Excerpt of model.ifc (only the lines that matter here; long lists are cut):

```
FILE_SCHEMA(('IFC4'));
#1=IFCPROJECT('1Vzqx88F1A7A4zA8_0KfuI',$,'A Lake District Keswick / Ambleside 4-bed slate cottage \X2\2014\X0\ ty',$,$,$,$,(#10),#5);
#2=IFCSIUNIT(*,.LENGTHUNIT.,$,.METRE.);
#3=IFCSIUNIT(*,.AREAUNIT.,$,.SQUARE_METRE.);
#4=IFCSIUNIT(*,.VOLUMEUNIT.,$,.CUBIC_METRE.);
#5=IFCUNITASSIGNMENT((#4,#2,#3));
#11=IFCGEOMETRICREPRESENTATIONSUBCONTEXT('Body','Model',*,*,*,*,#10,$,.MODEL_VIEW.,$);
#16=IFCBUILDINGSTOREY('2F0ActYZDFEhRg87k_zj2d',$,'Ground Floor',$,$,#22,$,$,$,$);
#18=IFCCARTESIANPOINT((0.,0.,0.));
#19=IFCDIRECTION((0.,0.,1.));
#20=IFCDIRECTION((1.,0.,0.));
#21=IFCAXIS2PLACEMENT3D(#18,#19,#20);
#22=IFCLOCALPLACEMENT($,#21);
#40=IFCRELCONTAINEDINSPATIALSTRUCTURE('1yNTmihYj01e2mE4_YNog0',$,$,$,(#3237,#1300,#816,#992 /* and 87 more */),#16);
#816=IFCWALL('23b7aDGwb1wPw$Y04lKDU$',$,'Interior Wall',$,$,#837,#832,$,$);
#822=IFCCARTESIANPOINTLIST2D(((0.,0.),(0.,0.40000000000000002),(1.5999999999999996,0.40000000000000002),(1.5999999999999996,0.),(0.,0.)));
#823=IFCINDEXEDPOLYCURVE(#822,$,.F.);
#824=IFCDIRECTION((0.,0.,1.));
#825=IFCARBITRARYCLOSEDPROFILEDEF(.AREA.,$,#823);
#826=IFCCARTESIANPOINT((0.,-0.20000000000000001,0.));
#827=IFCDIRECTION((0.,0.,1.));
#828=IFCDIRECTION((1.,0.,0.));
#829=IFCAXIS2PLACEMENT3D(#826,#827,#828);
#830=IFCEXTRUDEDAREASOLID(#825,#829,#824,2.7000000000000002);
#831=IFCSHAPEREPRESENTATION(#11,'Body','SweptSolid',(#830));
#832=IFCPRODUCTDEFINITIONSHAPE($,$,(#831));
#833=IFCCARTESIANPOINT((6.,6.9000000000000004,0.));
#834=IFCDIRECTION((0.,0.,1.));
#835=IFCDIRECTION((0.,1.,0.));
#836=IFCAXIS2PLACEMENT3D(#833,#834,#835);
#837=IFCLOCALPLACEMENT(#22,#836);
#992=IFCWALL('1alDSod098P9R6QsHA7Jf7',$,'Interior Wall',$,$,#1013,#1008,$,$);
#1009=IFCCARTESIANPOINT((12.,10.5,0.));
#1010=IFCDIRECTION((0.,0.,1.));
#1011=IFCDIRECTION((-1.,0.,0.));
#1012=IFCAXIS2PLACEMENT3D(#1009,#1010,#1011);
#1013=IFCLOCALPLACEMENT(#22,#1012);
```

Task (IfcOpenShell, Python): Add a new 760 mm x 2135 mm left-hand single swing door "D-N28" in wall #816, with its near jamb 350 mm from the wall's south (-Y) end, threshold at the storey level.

```python
import numpy as np
import ifcopenshell
import ifcopenshell.api.feature
import ifcopenshell.api.geometry
import ifcopenshell.api.root
import ifcopenshell.api.spatial
import ifcopenshell.geom
import ifcopenshell.util.element
import ifcopenshell.util.placement
import ifcopenshell.util.representation
import ifcopenshell.util.shape
import ifcopenshell.util.unit

model = ifcopenshell.open("model.ifc")
unit_scale = ifcopenshell.util.unit.calculate_unit_scale(model)
settings = ifcopenshell.geom.settings()


def volume(element):
    """Net volume in cubic metres, openings subtracted."""
    shape = ifcopenshell.geom.create_shape(settings, element)
    return ifcopenshell.util.shape.get_volume(shape.geometry)


wall = model.by_guid("23b7aDGwb1wPw$Y04lKDU$")
storey = ifcopenshell.util.element.get_container(wall, ifc_class="IfcBuildingStorey")
context = ifcopenshell.util.representation.get_context(model, "Model", "Body", "MODEL_VIEW")
before = volume(wall)

width, height, from_end, sill = 0.76, 2.135, 0.35, 0.0  # metres

# The wall runs along its own X axis, and the end named is its -X end.
wall_shape = ifcopenshell.geom.create_shape(settings, wall)
x, y, z = ifcopenshell.util.shape.get_vertices(wall_shape.geometry).T
start = x.min() + from_end
face, thickness = float(y.min()), float(y.max() - y.min())
wall_matrix = ifcopenshell.util.placement.get_local_placement(wall.ObjectPlacement)
level = ifcopenshell.util.placement.get_local_placement(storey.ObjectPlacement)[2, 3]


def in_wall(x, y):
    """Placement at x, y metres in the wall's axes, at sill height."""
    matrix = wall_matrix.copy()
    matrix[:, 3] = wall_matrix @ np.array([x / unit_scale, y / unit_scale, 0.0, 1.0])
    matrix[2, 3] = level + sill / unit_scale
    return matrix


# Opening: a box that overshoots both wall faces by 50 mm.
opening = ifcopenshell.api.root.create_entity(model, ifc_class="IfcOpeningElement", predefined_type="OPENING")
box = ifcopenshell.api.geometry.add_wall_representation(
    model, context=context, length=width, height=height, thickness=thickness + 0.1
)
ifcopenshell.api.geometry.assign_representation(model, product=opening, representation=box)
ifcopenshell.api.geometry.edit_object_placement(model, product=opening, matrix=in_wall(start, face - 0.05), is_si=False)
ifcopenshell.api.feature.add_feature(model, feature=opening, element=wall)

door = ifcopenshell.api.root.create_entity(model, ifc_class="IfcDoor", name="D-N28", predefined_type="DOOR")
door.OverallWidth, door.OverallHeight = width / unit_scale, height / unit_scale
door.OperationType = "SINGLE_SWING_LEFT"
body = ifcopenshell.api.geometry.add_door_representation(
    model,
    context=context,
    overall_width=door.OverallWidth,
    overall_height=door.OverallHeight,
    operation_type="SINGLE_SWING_LEFT",
    lining_properties={"LiningDepth": thickness / unit_scale, "ThresholdDepth": thickness / unit_scale},
)
ifcopenshell.api.geometry.assign_representation(model, product=door, representation=body)
ifcopenshell.api.spatial.assign_container(model, products=[door], relating_structure=storey)
ifcopenshell.api.feature.add_filling(model, opening=opening, element=door)

# The lining spans the wall, so the door starts at the wall face.
ifcopenshell.api.geometry.edit_object_placement(model, product=door, matrix=in_wall(start, face), is_si=False)

after = volume(wall)

print(f"wall volume {before:.3f} -> {after:.3f} m3")

model.write("model_rev.ifc")
```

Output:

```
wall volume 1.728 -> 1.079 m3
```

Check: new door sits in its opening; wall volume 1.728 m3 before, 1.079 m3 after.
